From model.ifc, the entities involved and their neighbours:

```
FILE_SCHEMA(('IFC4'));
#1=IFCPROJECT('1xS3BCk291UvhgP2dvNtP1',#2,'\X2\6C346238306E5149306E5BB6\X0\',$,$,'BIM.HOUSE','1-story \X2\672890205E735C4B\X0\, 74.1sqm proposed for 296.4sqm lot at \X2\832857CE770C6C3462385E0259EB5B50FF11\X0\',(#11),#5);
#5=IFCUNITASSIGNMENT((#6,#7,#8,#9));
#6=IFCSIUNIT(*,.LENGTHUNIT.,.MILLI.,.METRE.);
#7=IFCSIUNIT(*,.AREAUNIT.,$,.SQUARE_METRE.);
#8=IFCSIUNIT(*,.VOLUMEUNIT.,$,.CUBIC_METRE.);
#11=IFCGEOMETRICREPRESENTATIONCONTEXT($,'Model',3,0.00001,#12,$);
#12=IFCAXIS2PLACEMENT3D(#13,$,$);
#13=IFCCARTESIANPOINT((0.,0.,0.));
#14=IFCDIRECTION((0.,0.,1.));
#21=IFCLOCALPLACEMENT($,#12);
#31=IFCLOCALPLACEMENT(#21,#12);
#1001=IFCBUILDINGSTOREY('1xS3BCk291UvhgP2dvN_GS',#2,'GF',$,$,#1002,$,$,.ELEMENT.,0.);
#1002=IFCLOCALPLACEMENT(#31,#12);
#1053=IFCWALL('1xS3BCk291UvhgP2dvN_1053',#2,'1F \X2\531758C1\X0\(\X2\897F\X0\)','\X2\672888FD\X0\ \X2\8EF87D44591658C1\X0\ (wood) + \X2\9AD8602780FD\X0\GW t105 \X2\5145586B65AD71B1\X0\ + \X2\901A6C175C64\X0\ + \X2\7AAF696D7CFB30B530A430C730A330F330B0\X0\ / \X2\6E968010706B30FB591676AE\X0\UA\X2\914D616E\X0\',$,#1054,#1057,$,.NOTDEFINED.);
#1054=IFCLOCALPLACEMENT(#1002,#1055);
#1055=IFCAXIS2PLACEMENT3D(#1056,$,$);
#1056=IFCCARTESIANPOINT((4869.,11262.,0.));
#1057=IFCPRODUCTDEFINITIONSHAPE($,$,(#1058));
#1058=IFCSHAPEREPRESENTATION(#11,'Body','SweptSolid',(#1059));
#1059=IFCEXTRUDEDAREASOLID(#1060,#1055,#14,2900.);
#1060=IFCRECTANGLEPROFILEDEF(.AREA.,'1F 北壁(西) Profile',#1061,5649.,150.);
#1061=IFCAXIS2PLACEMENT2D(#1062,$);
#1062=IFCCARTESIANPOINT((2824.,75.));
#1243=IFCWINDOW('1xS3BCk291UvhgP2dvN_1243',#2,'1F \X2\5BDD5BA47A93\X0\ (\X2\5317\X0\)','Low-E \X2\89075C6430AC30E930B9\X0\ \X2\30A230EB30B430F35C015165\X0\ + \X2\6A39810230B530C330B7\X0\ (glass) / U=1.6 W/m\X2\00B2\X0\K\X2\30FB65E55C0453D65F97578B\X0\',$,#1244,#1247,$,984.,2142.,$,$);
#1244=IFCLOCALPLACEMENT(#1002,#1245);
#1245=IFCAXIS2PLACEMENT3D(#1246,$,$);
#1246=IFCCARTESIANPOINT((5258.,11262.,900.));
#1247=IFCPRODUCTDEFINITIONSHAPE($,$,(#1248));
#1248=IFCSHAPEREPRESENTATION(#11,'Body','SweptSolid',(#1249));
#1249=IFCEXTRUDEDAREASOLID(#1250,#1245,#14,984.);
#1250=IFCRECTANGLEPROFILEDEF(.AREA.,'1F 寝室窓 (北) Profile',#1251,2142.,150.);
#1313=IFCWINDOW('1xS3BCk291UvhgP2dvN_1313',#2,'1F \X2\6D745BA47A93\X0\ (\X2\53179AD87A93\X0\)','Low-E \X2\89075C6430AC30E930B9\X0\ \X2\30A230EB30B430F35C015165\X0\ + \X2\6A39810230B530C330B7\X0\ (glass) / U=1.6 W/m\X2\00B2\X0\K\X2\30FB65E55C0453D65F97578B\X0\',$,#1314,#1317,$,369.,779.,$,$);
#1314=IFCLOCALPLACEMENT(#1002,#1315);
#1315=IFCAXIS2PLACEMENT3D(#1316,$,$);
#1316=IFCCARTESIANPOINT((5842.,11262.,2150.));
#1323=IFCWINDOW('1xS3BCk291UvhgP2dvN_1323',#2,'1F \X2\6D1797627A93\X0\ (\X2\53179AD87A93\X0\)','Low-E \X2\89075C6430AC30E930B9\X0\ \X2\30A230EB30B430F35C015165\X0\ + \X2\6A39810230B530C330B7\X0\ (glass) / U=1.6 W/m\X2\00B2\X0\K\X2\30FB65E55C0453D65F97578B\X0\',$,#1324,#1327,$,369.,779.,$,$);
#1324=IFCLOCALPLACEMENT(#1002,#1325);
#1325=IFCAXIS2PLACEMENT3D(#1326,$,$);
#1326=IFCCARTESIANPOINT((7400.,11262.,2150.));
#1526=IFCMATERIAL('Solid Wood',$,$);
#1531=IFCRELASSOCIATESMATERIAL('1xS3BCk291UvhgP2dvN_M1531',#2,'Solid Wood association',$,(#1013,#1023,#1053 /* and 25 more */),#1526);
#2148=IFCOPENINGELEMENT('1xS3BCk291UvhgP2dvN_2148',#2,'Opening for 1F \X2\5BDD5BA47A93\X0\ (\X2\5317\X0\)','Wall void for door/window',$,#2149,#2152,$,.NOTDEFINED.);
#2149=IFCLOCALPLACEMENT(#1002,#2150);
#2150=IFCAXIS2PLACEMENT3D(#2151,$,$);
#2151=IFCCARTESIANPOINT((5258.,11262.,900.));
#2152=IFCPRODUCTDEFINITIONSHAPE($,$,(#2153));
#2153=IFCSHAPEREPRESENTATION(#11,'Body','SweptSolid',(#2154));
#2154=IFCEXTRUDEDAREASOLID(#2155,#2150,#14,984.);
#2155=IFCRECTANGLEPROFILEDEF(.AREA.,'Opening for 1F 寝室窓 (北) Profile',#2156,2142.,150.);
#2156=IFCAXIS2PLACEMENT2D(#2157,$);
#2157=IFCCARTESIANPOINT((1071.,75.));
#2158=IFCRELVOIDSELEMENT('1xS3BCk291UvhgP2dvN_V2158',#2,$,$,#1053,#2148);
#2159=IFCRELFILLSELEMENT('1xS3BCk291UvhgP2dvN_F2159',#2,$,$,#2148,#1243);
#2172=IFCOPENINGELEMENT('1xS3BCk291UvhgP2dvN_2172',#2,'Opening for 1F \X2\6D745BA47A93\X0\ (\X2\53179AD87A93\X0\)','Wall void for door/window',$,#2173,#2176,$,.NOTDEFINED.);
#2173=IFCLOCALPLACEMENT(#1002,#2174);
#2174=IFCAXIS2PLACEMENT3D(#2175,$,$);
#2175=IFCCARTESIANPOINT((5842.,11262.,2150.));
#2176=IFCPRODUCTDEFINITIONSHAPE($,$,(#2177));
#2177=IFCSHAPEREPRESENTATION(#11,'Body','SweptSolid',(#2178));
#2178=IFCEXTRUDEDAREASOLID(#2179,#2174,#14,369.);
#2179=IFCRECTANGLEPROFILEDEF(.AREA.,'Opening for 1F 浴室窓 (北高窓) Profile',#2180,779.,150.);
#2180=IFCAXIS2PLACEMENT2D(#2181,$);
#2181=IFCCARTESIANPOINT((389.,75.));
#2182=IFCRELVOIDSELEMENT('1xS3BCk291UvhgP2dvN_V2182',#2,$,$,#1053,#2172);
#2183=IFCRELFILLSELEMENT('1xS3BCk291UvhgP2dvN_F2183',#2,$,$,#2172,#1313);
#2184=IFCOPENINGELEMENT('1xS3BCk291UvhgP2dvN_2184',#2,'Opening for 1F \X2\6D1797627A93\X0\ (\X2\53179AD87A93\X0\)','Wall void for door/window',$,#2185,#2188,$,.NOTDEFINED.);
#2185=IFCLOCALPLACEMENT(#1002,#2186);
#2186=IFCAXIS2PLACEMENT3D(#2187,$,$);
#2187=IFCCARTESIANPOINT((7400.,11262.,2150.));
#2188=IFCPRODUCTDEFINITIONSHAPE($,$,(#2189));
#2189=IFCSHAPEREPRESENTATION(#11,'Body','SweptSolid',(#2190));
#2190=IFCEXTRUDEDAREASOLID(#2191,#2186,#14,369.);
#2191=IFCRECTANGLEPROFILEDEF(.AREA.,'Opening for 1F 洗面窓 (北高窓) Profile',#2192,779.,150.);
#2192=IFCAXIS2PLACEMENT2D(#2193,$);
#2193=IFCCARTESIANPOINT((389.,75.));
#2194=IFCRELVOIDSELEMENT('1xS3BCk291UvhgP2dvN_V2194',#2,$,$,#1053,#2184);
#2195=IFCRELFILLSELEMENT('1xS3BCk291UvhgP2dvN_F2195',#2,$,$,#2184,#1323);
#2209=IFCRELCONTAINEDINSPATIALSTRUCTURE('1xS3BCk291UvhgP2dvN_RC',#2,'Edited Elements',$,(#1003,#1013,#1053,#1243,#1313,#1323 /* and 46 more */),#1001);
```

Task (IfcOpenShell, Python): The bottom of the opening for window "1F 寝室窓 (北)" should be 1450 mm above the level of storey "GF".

```python
import numpy as np
import ifcopenshell
import ifcopenshell.api.geometry
import ifcopenshell.geom
import ifcopenshell.util.element
import ifcopenshell.util.placement
import ifcopenshell.util.shape
import ifcopenshell.util.unit

model = ifcopenshell.open("model.ifc")
unit_scale = ifcopenshell.util.unit.calculate_unit_scale(model)

window = model.by_guid("1xS3BCk291UvhgP2dvN_1243")
opening = window.FillsVoids[0].RelatingOpeningElement
storey = ifcopenshell.util.element.get_container(window, ifc_class="IfcBuildingStorey")
level = ifcopenshell.util.placement.get_local_placement(storey.ObjectPlacement)[2, 3]

# The opening's origin need not be at the sill, so measure its lowest point.
shape = ifcopenshell.geom.create_shape(ifcopenshell.geom.settings(), opening)
bottom = ifcopenshell.util.shape.get_shape_bottom_elevation(shape, shape.geometry) / unit_scale
dz = level + 1450.0 - bottom

shift = np.array([0.0, 0.0, dz])
# The window is not placed relative to its opening, so move both.
for product in (opening, window):
    matrix = ifcopenshell.util.placement.get_local_placement(product.ObjectPlacement)
    matrix[:3, 3] += shift
    ifcopenshell.api.geometry.edit_object_placement(model, product=product, matrix=matrix, is_si=False)

print(f"moved by {dz * unit_scale:+.3f} m")

model.write("model_edited.ifc")
```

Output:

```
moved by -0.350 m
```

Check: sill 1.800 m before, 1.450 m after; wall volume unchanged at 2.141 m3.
